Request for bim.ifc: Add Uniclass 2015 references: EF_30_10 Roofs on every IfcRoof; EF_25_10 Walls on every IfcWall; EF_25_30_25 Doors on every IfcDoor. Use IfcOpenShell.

First a look at what the model holds.

```python
import ifcopenshell

model = ifcopenshell.open("bim.ifc")
print(model.schema)
print("classifications:", [c.Name for c in model.by_type("IfcClassification")])
for ifc_class in ("IfcDoor", "IfcRoof", "IfcStair", "IfcWall", "IfcWindow"):
    print(ifc_class, len(model.by_type(ifc_class)))
```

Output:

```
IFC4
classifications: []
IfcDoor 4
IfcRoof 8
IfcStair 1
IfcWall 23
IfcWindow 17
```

```python
import ifcopenshell
import ifcopenshell.api.classification

model = ifcopenshell.open("bim.ifc")

system = ifcopenshell.api.classification.add_classification(model, classification="Uniclass 2015")

codes = {
    "IfcRoof": ("EF_30_10", "Roofs"),
    "IfcWall": ("EF_25_10", "Walls"),
    "IfcDoor": ("EF_25_30_25", "Doors"),
}
for ifc_class, (code, name) in codes.items():
    products = model.by_type(ifc_class)
    ifcopenshell.api.classification.add_reference(
        model, products=products, classification=system, identification=code, name=name
    )
    print(code, len(products))

model.write("bim_rev.ifc")
```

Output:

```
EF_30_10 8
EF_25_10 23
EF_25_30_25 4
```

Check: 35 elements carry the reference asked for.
